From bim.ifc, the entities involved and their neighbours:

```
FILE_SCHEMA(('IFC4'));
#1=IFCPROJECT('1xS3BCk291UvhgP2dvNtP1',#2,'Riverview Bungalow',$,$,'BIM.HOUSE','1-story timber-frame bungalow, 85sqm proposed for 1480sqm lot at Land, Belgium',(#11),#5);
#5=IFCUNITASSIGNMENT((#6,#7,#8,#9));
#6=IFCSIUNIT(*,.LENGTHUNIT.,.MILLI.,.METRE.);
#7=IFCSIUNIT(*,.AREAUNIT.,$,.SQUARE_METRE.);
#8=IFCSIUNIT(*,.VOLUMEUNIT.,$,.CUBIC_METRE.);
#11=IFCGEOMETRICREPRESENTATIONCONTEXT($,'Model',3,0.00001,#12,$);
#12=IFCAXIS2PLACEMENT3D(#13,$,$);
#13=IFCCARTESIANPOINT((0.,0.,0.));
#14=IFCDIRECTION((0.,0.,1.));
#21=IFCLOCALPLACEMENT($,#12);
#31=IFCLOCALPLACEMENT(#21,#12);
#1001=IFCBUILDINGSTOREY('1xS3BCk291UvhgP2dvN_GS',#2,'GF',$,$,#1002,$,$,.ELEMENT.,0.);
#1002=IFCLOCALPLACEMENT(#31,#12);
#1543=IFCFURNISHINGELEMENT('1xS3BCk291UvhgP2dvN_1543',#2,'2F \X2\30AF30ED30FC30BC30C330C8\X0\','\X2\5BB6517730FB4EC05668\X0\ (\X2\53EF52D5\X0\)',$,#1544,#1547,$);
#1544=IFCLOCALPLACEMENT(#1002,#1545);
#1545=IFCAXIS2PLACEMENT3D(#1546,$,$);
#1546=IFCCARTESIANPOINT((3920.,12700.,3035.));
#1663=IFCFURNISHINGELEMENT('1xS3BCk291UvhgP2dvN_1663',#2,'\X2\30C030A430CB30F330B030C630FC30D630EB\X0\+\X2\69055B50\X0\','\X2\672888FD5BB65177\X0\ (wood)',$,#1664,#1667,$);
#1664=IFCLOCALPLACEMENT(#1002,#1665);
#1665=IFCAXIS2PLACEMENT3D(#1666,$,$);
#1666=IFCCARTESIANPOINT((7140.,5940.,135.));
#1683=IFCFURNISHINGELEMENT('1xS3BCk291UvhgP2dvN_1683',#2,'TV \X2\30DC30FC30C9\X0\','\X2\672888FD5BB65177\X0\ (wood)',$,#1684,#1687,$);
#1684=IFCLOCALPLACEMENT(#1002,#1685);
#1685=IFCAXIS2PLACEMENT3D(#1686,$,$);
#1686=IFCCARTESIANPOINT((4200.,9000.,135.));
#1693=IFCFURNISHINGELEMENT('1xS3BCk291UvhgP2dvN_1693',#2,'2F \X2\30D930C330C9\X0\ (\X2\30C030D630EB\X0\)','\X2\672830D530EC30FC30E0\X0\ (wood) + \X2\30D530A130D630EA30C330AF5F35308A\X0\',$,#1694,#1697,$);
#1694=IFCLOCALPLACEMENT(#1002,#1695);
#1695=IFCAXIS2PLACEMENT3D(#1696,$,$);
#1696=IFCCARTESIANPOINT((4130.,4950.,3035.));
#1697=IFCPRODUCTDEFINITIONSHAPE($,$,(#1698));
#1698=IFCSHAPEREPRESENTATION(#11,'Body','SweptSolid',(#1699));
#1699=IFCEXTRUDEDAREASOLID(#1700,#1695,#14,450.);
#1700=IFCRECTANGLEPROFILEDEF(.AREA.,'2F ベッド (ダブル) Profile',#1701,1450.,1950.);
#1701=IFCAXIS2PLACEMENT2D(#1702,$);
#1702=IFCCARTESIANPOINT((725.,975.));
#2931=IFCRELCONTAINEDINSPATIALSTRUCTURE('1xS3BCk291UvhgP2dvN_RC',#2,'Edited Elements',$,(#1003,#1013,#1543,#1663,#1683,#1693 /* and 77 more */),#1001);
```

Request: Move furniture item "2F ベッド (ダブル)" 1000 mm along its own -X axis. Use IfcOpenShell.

```python
import ifcopenshell
import ifcopenshell.api.geometry
import ifcopenshell.util.placement

model = ifcopenshell.open("bim.ifc")

item = model.by_guid("1xS3BCk291UvhgP2dvN_1693")
matrix = ifcopenshell.util.placement.get_local_placement(item.ObjectPlacement)
matrix[:3, 3] -= matrix[:3, 0] * 1000.0
ifcopenshell.api.geometry.edit_object_placement(model, product=item, matrix=matrix, is_si=False)

print(ifcopenshell.util.placement.get_local_placement(item.ObjectPlacement).round(3) + 0.0)

model.write("bim_rev.ifc")
```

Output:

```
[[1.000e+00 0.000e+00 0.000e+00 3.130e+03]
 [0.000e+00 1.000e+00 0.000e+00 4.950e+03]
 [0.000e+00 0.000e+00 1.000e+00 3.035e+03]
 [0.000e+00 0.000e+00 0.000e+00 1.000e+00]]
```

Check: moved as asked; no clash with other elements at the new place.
